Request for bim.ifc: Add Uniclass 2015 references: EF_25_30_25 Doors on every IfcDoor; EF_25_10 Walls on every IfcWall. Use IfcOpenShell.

First a look at what the model holds.

```python
import ifcopenshell

model = ifcopenshell.open("bim.ifc")
print(model.schema)
print("classifications:", [c.Name for c in model.by_type("IfcClassification")])
for ifc_class in ("IfcDoor", "IfcRoof", "IfcStair", "IfcWall", "IfcWindow"):
    print(ifc_class, len(model.by_type(ifc_class)))
```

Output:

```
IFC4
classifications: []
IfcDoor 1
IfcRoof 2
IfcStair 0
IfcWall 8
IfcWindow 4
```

```python
import ifcopenshell
import ifcopenshell.api.classification

model = ifcopenshell.open("bim.ifc")

system = ifcopenshell.api.classification.add_classification(model, classification="Uniclass 2015")

codes = {
    "IfcDoor": ("EF_25_30_25", "Doors"),
    "IfcWall": ("EF_25_10", "Walls"),
}
for ifc_class, (code, name) in codes.items():
    products = model.by_type(ifc_class)
    ifcopenshell.api.classification.add_reference(
        model, products=products, classification=system, identification=code, name=name
    )
    print(code, len(products))

model.write("bim_rev.ifc")
```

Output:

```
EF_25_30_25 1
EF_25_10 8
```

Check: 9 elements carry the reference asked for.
